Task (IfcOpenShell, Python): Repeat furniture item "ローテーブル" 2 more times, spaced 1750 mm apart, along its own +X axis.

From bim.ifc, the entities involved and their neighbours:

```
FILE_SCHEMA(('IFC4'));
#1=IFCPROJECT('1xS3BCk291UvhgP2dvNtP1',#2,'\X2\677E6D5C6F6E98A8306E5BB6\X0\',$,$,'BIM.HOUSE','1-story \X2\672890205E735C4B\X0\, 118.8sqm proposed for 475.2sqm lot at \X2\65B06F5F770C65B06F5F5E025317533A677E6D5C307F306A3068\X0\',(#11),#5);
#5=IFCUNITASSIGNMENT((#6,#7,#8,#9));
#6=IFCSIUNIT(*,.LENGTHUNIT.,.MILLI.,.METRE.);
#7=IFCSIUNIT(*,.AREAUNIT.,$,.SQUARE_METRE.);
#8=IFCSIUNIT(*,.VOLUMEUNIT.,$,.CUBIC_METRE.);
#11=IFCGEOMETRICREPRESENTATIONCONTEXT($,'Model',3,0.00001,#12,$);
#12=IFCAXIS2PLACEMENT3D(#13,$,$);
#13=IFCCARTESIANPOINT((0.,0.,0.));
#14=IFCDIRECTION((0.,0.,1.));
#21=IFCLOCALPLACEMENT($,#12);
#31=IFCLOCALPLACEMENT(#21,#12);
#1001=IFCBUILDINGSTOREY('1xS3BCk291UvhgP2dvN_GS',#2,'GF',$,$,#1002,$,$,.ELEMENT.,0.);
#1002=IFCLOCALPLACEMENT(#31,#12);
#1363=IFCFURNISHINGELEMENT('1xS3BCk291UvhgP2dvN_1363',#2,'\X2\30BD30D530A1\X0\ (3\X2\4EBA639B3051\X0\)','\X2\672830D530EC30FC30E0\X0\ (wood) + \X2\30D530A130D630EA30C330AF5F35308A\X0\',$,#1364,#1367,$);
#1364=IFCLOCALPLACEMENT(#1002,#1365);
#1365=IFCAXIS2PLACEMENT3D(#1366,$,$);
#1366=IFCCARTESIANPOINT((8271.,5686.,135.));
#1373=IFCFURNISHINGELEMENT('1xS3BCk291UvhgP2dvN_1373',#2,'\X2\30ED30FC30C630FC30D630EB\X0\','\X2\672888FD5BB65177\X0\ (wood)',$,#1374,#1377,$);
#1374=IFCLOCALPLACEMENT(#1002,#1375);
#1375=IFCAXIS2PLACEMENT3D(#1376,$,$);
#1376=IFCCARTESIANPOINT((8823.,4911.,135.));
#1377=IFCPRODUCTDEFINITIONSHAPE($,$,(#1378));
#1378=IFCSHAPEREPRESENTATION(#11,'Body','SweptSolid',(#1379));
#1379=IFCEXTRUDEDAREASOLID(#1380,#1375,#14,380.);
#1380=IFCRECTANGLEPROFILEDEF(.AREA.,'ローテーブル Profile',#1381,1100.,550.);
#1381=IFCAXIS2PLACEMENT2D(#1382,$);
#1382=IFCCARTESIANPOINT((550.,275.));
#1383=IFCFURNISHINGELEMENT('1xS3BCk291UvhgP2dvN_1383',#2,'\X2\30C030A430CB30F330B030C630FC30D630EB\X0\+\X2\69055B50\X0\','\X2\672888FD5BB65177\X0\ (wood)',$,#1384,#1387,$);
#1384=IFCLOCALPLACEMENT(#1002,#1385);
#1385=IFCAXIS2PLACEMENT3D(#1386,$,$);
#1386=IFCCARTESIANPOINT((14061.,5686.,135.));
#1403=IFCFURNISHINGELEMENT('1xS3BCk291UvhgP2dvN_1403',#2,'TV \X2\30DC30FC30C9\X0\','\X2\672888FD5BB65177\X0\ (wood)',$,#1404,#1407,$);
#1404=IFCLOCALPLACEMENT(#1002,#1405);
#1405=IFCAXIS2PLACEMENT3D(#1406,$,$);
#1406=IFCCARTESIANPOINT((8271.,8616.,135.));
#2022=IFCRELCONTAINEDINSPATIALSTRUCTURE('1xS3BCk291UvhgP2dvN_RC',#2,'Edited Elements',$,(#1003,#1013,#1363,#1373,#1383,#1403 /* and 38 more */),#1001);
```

```python
import ifcopenshell
import ifcopenshell.api.geometry
import ifcopenshell.api.root
import ifcopenshell.util.element
import ifcopenshell.util.placement
import ifcopenshell.util.unit

model = ifcopenshell.open("bim.ifc")
unit_scale = ifcopenshell.util.unit.calculate_unit_scale(model)


def reuse_history(source, copy):
    """copy_class also copies each property set's owner history, people and application; keep the originals."""
    for rel in copy.IsDefinedBy:
        if rel.is_a("IfcRelDefinesByProperties") and (history := rel.RelatingPropertyDefinition.OwnerHistory):
            rel.RelatingPropertyDefinition.OwnerHistory = source.OwnerHistory
            ifcopenshell.util.element.remove_deep2(model, history)


source = model.by_guid("1xS3BCk291UvhgP2dvN_1373")
base = ifcopenshell.util.placement.get_local_placement(source.ObjectPlacement)
step = base[:3, 0] * 1.75 / unit_scale

for i in range(1, 3):
    copy = ifcopenshell.api.root.copy_class(model, product=source)
    copy.Representation = ifcopenshell.util.element.copy_deep(
        model, source.Representation, exclude=["IfcGeometricRepresentationContext", "IfcRepresentationMap"]
    )
    reuse_history(source, copy)
    matrix = base.copy()
    matrix[:3, 3] += i * step
    print("added at", matrix[:3, 3].round(3) + 0.0)
    ifcopenshell.api.geometry.edit_object_placement(model, product=copy, matrix=matrix, is_si=False)

model.write("bim_rev.ifc")
```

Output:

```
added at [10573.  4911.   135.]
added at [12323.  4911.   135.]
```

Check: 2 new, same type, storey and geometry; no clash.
